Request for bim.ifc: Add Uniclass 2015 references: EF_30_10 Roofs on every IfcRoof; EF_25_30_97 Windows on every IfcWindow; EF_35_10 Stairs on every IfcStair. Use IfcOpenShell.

First a look at what the model holds.

```python
import ifcopenshell

model = ifcopenshell.open("bim.ifc")
print(model.schema)
print("classifications:", [c.Name for c in model.by_type("IfcClassification")])
for ifc_class in ("IfcDoor", "IfcRoof", "IfcStair", "IfcWall", "IfcWindow"):
    print(ifc_class, len(model.by_type(ifc_class)))
```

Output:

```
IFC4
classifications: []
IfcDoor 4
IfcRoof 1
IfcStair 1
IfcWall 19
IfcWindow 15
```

```python
import ifcopenshell
import ifcopenshell.api.classification

model = ifcopenshell.open("bim.ifc")

system = ifcopenshell.api.classification.add_classification(model, classification="Uniclass 2015")

codes = {
    "IfcRoof": ("EF_30_10", "Roofs"),
    "IfcWindow": ("EF_25_30_97", "Windows"),
    "IfcStair": ("EF_35_10", "Stairs"),
}
for ifc_class, (code, name) in codes.items():
    products = model.by_type(ifc_class)
    ifcopenshell.api.classification.add_reference(
        model, products=products, classification=system, identification=code, name=name
    )
    print(code, len(products))

model.write("bim_edited.ifc")
```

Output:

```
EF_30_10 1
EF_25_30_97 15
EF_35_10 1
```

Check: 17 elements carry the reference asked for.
